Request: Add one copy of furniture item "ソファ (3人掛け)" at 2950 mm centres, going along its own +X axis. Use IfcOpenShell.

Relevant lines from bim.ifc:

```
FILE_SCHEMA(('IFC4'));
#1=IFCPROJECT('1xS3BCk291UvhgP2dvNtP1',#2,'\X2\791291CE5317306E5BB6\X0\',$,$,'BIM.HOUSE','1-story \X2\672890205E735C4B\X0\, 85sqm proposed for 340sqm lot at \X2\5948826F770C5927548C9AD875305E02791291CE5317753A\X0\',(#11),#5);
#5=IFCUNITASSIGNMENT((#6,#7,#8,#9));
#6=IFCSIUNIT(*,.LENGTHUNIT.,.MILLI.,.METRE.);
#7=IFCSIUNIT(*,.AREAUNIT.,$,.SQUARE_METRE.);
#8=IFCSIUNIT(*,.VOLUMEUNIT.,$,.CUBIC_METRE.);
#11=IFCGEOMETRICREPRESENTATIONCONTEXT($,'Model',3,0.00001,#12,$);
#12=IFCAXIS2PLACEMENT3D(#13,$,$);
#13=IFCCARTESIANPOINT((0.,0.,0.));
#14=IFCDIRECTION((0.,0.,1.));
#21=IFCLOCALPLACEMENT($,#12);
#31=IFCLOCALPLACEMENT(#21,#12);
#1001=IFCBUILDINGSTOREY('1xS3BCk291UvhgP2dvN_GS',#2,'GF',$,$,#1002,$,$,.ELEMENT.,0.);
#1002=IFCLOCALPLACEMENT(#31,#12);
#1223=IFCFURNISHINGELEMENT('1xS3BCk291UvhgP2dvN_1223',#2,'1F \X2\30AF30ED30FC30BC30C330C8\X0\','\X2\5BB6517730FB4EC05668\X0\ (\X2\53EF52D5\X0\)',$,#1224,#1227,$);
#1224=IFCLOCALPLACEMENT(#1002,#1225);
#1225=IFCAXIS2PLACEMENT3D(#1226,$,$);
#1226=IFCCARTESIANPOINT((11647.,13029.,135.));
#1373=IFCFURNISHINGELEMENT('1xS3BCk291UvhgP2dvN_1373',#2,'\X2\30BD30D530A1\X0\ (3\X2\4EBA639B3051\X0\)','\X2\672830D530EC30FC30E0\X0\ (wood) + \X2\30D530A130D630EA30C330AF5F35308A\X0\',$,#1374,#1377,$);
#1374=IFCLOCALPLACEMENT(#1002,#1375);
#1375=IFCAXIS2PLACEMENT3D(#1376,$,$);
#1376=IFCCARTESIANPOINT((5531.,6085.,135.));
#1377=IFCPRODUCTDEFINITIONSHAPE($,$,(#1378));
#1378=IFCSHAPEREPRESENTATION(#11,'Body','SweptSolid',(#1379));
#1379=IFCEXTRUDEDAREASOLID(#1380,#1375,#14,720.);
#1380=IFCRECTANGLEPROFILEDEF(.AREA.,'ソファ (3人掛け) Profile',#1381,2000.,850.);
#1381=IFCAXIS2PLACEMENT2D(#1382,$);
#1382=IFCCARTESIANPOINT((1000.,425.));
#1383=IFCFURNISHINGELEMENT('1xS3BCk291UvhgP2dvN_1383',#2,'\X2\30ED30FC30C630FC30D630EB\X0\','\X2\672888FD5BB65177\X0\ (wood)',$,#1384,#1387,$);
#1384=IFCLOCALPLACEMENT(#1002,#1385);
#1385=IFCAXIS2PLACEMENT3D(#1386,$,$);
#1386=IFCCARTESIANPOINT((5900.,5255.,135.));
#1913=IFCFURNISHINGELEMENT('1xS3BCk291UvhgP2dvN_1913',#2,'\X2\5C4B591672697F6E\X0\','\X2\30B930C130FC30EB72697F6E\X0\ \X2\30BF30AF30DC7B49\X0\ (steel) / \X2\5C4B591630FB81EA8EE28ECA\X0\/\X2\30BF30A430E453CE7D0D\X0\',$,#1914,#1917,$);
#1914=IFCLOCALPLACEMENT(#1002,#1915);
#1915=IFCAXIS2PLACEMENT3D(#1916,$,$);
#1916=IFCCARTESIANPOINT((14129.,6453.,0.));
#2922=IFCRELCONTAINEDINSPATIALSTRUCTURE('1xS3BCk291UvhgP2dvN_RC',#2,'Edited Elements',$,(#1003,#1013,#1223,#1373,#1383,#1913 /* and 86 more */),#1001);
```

```python
import ifcopenshell
import ifcopenshell.api.geometry
import ifcopenshell.api.root
import ifcopenshell.util.element
import ifcopenshell.util.placement
import ifcopenshell.util.unit

model = ifcopenshell.open("bim.ifc")
unit_scale = ifcopenshell.util.unit.calculate_unit_scale(model)


def reuse_history(source, copy):
    """copy_class also copies each property set's owner history, people and application; keep the originals."""
    for rel in copy.IsDefinedBy:
        if rel.is_a("IfcRelDefinesByProperties") and (history := rel.RelatingPropertyDefinition.OwnerHistory):
            rel.RelatingPropertyDefinition.OwnerHistory = source.OwnerHistory
            ifcopenshell.util.element.remove_deep2(model, history)


source = model.by_guid("1xS3BCk291UvhgP2dvN_1373")
base = ifcopenshell.util.placement.get_local_placement(source.ObjectPlacement)
step = base[:3, 0] * 2.95 / unit_scale

for i in range(1, 2):
    copy = ifcopenshell.api.root.copy_class(model, product=source)
    copy.Representation = ifcopenshell.util.element.copy_deep(
        model, source.Representation, exclude=["IfcGeometricRepresentationContext", "IfcRepresentationMap"]
    )
    reuse_history(source, copy)
    matrix = base.copy()
    matrix[:3, 3] += i * step
    print("added at", matrix[:3, 3].round(3) + 0.0)
    ifcopenshell.api.geometry.edit_object_placement(model, product=copy, matrix=matrix, is_si=False)

model.write("bim_rev.ifc")
```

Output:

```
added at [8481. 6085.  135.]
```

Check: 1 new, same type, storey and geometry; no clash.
